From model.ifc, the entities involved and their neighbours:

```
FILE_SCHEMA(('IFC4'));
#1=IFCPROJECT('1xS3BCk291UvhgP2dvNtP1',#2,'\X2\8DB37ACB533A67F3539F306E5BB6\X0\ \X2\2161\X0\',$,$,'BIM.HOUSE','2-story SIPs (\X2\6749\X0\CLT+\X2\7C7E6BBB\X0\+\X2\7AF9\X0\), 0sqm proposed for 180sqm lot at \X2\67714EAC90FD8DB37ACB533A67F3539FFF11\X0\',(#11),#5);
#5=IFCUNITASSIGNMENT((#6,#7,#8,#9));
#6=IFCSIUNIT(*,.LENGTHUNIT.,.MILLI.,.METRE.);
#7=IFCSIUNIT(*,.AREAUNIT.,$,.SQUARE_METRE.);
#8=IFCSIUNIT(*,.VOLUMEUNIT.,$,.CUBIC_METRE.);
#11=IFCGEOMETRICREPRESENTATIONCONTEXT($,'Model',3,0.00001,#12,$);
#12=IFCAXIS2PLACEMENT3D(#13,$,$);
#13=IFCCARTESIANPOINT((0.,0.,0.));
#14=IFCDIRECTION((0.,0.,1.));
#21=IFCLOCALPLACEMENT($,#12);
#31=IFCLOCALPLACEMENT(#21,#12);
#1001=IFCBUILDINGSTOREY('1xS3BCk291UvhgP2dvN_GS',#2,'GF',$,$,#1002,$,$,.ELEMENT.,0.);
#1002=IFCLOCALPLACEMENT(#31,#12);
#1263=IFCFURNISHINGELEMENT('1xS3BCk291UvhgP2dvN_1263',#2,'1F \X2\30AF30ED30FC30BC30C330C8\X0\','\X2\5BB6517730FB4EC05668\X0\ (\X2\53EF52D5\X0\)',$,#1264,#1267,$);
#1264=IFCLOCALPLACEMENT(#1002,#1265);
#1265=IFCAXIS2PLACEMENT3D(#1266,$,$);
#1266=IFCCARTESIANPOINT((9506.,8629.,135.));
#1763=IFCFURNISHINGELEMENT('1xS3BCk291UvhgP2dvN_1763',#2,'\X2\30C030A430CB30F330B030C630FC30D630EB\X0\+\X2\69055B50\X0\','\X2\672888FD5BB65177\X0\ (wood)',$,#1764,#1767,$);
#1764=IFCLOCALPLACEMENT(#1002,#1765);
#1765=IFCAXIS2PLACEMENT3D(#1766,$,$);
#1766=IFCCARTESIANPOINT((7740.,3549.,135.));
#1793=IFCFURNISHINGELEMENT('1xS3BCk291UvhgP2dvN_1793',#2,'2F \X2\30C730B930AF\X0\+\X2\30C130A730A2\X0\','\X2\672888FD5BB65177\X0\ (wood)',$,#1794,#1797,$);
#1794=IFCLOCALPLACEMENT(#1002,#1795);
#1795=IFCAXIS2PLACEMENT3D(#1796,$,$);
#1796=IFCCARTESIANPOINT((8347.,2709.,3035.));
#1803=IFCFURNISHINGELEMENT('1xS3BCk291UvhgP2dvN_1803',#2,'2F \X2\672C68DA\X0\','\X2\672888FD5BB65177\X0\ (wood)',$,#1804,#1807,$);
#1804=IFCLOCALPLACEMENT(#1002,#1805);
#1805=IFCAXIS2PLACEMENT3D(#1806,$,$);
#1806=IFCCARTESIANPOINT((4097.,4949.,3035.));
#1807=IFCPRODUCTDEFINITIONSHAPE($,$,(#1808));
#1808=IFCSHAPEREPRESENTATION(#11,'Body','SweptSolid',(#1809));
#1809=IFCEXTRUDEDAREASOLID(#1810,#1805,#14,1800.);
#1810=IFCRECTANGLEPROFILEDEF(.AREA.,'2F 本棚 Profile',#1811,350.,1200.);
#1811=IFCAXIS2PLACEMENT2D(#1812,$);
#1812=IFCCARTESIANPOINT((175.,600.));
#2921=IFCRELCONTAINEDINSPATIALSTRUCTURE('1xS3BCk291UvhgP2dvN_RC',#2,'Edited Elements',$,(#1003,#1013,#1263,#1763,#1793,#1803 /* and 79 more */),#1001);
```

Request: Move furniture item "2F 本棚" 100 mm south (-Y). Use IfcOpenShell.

```python
import ifcopenshell
import ifcopenshell.api.geometry
import ifcopenshell.util.placement
import ifcopenshell.util.unit

model = ifcopenshell.open("model.ifc")
unit_scale = ifcopenshell.util.unit.calculate_unit_scale(model)

item = model.by_guid("1xS3BCk291UvhgP2dvN_1803")
matrix = ifcopenshell.util.placement.get_local_placement(item.ObjectPlacement)
matrix[1, 3] -= 0.1 / unit_scale
ifcopenshell.api.geometry.edit_object_placement(model, product=item, matrix=matrix, is_si=False)

print(ifcopenshell.util.placement.get_local_placement(item.ObjectPlacement).round(3) + 0.0)

model.write("model_v2.ifc")
```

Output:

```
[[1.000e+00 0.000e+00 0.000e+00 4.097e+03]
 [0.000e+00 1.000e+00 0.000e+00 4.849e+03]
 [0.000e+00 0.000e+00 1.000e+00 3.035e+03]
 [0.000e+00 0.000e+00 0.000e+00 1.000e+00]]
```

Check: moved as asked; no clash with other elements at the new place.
